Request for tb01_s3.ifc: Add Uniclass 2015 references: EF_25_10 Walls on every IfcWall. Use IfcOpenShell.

First a look at what the model holds.

```python
import ifcopenshell

model = ifcopenshell.open("tb01_s3.ifc")
print(model.schema)
print("classifications:", [c.Name for c in model.by_type("IfcClassification")])
for ifc_class in ("IfcDoor", "IfcRoof", "IfcStair", "IfcWall", "IfcWindow"):
    print(ifc_class, len(model.by_type(ifc_class)))
```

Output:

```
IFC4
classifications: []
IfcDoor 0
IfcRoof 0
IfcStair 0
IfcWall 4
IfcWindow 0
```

```python
import ifcopenshell
import ifcopenshell.api.classification

model = ifcopenshell.open("tb01_s3.ifc")

system = ifcopenshell.api.classification.add_classification(model, classification="Uniclass 2015")

codes = {
    "IfcWall": ("EF_25_10", "Walls"),
}
for ifc_class, (code, name) in codes.items():
    products = model.by_type(ifc_class)
    ifcopenshell.api.classification.add_reference(
        model, products=products, classification=system, identification=code, name=name
    )
    print(code, len(products))

model.write("tb01_s3_edited.ifc")
```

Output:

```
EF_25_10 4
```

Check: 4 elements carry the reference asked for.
